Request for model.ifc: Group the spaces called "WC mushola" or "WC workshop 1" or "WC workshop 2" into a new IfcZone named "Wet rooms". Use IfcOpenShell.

First a look at what the model holds.

```python
import ifcopenshell

model = ifcopenshell.open("model.ifc")
print(model.schema)
seen = {}
for space in model.by_type("IfcSpace"):
    seen[space.Name] = seen.get(space.Name, 0) + 1
for name, count in sorted(seen.items(), key=str):
    print(count, "x", name)
print("zones:", [z.Name for z in model.by_type("IfcZone")][:20])
```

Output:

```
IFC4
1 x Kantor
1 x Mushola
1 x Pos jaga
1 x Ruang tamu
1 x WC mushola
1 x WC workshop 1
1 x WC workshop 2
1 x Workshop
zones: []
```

```python
import ifcopenshell
import ifcopenshell.api.group
import ifcopenshell.api.root

model = ifcopenshell.open("model.ifc")

names = {"WC mushola", "WC workshop 1", "WC workshop 2"}
spaces = [s for s in model.by_type("IfcSpace") if s.Name in names]

zone = ifcopenshell.api.root.create_entity(model, ifc_class="IfcZone", name="Wet rooms")
ifcopenshell.api.group.assign_group(model, products=spaces, group=zone)
print(len(spaces), "spaces in", zone.Name)

model.write("model_edited.ifc")
```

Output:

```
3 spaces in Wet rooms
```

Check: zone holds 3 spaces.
